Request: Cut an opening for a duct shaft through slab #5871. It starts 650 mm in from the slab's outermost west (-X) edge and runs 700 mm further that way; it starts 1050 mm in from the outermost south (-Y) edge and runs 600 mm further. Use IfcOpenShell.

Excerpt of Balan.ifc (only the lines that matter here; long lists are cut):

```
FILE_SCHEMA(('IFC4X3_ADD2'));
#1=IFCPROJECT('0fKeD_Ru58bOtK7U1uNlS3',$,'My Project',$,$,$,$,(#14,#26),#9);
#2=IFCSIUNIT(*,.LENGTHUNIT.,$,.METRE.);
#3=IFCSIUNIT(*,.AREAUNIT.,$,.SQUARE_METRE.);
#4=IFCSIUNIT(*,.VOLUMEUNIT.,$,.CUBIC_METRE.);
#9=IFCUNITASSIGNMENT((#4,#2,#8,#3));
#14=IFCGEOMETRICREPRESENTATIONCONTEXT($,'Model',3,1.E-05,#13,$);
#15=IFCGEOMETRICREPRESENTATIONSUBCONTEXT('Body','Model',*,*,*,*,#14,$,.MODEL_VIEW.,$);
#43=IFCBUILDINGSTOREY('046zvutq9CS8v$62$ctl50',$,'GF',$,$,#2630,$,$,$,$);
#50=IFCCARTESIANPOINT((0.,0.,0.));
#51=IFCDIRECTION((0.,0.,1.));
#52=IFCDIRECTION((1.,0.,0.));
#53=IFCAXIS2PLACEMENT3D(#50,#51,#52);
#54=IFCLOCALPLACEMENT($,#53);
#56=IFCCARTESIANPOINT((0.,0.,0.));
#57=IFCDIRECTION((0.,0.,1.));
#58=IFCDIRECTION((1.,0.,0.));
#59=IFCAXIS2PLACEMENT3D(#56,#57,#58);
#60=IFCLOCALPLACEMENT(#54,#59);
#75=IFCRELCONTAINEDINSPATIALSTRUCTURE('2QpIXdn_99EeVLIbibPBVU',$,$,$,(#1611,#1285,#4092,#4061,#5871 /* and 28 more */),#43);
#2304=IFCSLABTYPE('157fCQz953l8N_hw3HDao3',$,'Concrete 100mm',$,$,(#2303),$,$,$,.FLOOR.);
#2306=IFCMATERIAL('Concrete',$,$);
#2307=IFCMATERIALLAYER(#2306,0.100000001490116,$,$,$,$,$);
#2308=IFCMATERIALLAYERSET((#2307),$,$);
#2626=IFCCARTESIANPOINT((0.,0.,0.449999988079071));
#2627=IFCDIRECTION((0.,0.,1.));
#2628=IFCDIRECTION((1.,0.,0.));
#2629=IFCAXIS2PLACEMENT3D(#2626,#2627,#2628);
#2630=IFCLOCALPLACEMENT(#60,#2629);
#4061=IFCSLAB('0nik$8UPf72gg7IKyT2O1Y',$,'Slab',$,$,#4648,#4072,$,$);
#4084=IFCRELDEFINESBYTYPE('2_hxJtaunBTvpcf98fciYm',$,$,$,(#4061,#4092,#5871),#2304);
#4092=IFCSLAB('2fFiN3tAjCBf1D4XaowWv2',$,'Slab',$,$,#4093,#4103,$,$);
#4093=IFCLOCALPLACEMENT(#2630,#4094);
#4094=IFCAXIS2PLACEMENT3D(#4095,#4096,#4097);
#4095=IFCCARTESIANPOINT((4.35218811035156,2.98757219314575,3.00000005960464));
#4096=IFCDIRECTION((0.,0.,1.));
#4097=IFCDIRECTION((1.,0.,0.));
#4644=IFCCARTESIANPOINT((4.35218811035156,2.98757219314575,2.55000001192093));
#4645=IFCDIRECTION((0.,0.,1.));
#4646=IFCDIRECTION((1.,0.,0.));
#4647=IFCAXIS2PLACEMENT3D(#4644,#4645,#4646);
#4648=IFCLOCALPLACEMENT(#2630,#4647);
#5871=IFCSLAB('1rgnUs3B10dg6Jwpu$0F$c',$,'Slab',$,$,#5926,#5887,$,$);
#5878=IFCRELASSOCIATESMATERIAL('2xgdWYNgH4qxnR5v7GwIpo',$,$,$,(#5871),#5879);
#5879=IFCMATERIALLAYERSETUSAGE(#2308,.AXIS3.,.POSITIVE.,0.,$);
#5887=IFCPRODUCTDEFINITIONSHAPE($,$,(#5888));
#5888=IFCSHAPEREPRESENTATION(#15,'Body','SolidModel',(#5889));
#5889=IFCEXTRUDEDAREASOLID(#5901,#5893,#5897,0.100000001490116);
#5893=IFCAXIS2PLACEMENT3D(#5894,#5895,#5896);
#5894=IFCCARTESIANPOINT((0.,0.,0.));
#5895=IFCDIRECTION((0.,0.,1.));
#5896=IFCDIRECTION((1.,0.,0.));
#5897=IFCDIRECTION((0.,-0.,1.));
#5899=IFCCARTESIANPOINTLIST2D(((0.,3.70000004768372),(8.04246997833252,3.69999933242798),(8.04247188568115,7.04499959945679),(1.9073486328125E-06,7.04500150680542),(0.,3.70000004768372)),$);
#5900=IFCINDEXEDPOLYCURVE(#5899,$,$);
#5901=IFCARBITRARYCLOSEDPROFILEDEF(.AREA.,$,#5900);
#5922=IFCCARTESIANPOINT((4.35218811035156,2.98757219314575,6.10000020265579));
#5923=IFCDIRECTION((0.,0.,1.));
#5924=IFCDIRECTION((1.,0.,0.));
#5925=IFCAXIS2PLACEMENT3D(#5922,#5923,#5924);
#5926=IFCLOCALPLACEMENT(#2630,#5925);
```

```python
import numpy as np
import ifcopenshell
import ifcopenshell.api.feature
import ifcopenshell.api.geometry
import ifcopenshell.api.root
import ifcopenshell.geom
import ifcopenshell.util.placement
import ifcopenshell.util.representation
import ifcopenshell.util.shape
import ifcopenshell.util.unit

model = ifcopenshell.open("Balan.ifc")
unit_scale = ifcopenshell.util.unit.calculate_unit_scale(model)
settings = ifcopenshell.geom.settings()


def volume(element):
    """Net volume in cubic metres, openings subtracted."""
    shape = ifcopenshell.geom.create_shape(settings, element)
    return ifcopenshell.util.shape.get_volume(shape.geometry)


slab = model.by_id(5871)
before = volume(slab)

# Extent in the slab's own axes, in metres. The edges named are its -X and -Y sides.
slab_shape = ifcopenshell.geom.create_shape(settings, slab)
vertices = ifcopenshell.util.shape.get_vertices(slab_shape.geometry)
x_min, y_min, bottom = vertices.min(axis=0)
top = vertices[:, 2].max()

opening = ifcopenshell.api.root.create_entity(model, ifc_class="IfcOpeningElement", name="Duct shaft opening", predefined_type="OPENING")
context = ifcopenshell.util.representation.get_context(model, "Model", "Body", "MODEL_VIEW")
width, depth = 0.7, 0.6
outline = [(0.0, 0.0), (width, 0.0), (width, depth), (0.0, depth), (0.0, 0.0)]
# Overshoot both faces by 50 mm so the cut is clean.
shape = ifcopenshell.api.geometry.add_slab_representation(
    model, context=context, depth=top - bottom + 0.1, polyline=outline
)
ifcopenshell.api.geometry.assign_representation(model, product=opening, representation=shape)

matrix = ifcopenshell.util.placement.get_local_placement(slab.ObjectPlacement)
matrix[:, 3] = matrix @ np.append(np.array([x_min + 0.65, y_min + 1.05, bottom - 0.05]) / unit_scale, 1.0)
ifcopenshell.api.geometry.edit_object_placement(model, product=opening, matrix=matrix, is_si=False)
ifcopenshell.api.feature.add_feature(model, feature=opening, element=slab)

after = volume(slab)

print(f"slab volume {before:.3f} -> {after:.3f} m3")

model.write("Balan_updated.ifc")
```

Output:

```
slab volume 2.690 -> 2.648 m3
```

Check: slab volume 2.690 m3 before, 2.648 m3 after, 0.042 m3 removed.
